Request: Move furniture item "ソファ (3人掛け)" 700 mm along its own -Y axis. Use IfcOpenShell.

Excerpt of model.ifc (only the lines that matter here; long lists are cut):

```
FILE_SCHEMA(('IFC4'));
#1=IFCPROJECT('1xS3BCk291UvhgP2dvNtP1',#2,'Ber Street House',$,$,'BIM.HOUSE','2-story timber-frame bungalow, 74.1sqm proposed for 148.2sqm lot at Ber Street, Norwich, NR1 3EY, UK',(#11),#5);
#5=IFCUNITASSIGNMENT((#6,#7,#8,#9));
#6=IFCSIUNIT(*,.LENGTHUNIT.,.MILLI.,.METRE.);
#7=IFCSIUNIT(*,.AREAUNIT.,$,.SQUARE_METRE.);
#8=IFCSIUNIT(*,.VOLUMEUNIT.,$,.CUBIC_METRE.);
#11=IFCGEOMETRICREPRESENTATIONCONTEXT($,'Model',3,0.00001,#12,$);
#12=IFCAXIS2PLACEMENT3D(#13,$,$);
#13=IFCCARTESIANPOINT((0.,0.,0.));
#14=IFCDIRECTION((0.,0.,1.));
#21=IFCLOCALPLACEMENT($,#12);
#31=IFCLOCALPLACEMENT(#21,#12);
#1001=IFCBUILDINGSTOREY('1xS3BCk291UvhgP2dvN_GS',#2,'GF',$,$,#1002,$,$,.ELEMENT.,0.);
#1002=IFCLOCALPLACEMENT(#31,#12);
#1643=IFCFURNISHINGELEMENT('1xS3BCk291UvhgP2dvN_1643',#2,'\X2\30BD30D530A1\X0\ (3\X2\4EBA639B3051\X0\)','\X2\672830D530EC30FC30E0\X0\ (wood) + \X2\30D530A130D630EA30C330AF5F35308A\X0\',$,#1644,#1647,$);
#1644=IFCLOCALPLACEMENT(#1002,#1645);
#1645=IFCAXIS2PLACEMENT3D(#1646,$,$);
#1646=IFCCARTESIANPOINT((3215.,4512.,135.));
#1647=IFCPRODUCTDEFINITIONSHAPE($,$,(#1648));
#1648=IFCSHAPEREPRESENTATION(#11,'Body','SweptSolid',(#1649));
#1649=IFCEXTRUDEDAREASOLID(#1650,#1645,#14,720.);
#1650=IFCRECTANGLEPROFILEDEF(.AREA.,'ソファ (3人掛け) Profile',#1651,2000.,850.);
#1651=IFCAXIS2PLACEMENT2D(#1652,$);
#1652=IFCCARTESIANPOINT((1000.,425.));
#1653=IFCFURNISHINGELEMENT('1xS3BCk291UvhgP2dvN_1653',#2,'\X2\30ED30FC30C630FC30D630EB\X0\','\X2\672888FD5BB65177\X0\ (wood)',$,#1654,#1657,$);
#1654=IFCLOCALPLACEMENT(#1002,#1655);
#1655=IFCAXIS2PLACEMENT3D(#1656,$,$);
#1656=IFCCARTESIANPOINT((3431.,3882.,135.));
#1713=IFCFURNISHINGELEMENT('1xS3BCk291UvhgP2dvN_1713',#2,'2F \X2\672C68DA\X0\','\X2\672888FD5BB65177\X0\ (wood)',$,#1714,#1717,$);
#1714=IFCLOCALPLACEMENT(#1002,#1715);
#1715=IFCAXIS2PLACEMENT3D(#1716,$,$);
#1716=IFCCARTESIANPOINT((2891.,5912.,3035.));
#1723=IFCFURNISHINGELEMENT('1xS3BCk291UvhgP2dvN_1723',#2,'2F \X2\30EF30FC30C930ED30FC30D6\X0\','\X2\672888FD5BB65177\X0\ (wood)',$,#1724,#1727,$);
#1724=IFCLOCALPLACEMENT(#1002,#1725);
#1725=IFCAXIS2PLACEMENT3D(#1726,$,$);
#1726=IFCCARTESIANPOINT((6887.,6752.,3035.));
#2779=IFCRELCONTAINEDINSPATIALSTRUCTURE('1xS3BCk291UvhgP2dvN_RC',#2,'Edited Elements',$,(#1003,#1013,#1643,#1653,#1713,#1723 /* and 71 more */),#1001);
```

```python
import ifcopenshell
import ifcopenshell.api.geometry
import ifcopenshell.util.placement
import ifcopenshell.util.unit

model = ifcopenshell.open("model.ifc")
unit_scale = ifcopenshell.util.unit.calculate_unit_scale(model)

item = model.by_guid("1xS3BCk291UvhgP2dvN_1643")
matrix = ifcopenshell.util.placement.get_local_placement(item.ObjectPlacement)
matrix[:3, 3] -= matrix[:3, 1] * 0.7 / unit_scale
ifcopenshell.api.geometry.edit_object_placement(model, product=item, matrix=matrix, is_si=False)

print(ifcopenshell.util.placement.get_local_placement(item.ObjectPlacement).round(3) + 0.0)

model.write("model_v2.ifc")
```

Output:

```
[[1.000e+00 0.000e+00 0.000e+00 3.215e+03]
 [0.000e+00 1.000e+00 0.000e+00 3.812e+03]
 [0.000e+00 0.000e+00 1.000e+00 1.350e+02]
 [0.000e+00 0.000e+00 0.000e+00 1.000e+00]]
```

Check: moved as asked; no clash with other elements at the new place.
